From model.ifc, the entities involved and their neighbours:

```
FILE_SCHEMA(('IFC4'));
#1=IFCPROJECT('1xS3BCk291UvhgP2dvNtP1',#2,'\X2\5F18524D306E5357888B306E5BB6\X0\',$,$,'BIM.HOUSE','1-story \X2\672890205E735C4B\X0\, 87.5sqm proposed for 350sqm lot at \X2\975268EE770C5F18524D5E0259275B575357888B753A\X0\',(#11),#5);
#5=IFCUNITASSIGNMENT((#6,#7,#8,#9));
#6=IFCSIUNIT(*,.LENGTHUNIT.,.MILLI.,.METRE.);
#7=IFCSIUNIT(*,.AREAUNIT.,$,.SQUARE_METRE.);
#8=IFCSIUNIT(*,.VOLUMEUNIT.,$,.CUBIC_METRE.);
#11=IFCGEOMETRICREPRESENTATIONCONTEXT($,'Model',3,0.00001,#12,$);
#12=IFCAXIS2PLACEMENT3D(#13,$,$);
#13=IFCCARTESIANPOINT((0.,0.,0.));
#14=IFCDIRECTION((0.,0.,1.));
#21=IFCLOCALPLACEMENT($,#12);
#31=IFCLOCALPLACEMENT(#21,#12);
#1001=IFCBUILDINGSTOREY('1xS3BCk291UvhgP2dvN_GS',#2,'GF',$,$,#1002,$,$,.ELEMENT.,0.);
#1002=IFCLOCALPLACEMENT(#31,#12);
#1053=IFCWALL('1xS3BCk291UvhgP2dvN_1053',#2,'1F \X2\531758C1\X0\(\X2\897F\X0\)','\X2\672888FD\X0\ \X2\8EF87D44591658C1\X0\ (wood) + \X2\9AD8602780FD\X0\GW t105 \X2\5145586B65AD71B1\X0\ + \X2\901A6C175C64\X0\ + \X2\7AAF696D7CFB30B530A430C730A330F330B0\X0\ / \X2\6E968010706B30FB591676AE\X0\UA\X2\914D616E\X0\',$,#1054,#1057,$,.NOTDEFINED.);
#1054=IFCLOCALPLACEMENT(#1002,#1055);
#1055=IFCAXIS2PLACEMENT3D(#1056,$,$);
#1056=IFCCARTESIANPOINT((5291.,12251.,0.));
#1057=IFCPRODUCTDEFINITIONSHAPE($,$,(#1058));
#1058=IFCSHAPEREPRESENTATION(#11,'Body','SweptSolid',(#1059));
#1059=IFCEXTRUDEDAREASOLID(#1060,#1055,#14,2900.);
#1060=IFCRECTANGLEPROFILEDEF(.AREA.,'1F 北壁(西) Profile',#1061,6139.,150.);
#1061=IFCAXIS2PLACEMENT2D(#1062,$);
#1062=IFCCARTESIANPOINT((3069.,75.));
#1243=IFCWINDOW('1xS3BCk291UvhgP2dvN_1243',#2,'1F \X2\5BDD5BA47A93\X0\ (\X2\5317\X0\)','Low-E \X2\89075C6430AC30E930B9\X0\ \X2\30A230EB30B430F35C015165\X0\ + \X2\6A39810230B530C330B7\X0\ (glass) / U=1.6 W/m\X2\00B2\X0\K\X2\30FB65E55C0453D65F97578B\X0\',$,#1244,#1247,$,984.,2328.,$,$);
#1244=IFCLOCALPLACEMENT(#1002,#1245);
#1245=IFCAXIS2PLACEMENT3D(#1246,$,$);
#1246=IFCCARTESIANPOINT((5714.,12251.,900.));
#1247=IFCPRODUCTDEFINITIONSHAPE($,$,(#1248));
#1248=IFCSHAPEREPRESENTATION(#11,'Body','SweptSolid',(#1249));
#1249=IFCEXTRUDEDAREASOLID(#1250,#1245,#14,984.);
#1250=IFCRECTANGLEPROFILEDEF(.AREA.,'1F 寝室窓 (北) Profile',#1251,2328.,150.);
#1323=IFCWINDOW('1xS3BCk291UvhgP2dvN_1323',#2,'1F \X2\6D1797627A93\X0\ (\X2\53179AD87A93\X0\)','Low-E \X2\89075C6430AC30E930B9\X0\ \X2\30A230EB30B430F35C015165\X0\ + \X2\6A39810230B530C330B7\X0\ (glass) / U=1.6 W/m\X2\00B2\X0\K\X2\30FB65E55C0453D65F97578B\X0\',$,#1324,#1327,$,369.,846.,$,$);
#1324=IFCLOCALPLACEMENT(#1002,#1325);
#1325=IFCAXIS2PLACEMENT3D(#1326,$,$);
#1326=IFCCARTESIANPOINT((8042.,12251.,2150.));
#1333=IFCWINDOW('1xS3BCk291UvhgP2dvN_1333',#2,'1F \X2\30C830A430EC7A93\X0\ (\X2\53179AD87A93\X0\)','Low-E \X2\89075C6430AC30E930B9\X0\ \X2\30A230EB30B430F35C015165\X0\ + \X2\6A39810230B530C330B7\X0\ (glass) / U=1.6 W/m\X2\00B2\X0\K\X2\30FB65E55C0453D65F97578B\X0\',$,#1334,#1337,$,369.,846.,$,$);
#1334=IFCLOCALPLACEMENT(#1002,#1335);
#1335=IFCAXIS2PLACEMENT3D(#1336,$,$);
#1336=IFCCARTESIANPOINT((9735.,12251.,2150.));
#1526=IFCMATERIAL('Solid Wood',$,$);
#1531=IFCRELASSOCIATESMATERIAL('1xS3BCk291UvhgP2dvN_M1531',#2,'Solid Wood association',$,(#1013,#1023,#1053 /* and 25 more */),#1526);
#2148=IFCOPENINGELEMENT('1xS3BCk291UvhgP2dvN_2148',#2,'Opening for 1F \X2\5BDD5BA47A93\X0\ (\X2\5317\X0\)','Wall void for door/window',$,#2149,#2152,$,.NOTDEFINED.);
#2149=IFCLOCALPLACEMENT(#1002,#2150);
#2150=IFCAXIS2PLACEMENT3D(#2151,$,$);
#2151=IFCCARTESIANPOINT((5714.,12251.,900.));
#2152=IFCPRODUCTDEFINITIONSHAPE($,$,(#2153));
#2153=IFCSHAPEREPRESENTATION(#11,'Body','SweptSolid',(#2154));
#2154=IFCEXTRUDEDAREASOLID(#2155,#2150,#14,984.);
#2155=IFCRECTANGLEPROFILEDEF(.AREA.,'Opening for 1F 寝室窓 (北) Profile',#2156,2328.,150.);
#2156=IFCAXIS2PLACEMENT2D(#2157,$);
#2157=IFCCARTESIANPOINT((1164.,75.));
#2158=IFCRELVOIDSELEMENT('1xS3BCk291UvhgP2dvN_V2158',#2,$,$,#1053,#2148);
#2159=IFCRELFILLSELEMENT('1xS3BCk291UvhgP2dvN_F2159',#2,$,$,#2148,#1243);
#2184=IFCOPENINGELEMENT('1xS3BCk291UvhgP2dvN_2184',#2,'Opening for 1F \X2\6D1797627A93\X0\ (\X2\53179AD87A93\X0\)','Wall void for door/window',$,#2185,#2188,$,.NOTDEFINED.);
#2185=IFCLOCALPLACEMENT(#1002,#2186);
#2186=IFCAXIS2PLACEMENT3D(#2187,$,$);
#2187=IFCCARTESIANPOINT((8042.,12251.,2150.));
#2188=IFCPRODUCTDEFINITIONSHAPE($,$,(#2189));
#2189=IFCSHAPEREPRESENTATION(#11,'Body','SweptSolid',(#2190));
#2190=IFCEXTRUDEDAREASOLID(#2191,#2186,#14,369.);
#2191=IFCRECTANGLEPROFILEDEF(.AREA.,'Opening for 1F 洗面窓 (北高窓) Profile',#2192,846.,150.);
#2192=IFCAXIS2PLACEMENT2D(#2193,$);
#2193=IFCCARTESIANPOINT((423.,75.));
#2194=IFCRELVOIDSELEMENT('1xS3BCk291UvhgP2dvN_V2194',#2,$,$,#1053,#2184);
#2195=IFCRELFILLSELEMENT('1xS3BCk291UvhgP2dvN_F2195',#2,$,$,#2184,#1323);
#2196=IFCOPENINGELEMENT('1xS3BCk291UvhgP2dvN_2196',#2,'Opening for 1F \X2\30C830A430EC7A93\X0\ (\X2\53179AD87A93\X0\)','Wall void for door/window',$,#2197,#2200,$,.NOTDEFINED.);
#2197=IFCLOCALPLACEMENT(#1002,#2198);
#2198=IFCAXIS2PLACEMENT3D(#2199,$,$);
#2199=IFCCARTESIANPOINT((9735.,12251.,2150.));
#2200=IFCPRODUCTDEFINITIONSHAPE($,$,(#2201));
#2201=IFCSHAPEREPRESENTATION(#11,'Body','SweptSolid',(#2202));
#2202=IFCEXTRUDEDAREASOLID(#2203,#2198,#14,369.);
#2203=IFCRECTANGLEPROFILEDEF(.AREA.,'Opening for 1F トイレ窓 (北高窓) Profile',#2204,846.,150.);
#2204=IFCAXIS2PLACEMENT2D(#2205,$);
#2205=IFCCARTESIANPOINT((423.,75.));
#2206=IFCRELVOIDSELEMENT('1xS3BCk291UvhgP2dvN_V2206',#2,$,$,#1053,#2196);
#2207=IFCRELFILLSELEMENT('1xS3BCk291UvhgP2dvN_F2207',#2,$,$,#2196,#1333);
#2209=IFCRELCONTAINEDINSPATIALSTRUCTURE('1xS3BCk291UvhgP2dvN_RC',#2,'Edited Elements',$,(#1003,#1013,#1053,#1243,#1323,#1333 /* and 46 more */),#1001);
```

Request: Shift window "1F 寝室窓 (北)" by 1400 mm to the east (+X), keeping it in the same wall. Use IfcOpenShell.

```python
import ifcopenshell
import ifcopenshell.api.geometry
import ifcopenshell.util.placement

model = ifcopenshell.open("model.ifc")

window = model.by_guid("1xS3BCk291UvhgP2dvN_1243")
opening = window.FillsVoids[0].RelatingOpeningElement
wall = opening.VoidsElements[0].RelatingBuildingElement

wall_matrix = ifcopenshell.util.placement.get_local_placement(wall.ObjectPlacement)
shift = wall_matrix[:3, 0] * 1400.0
before = ifcopenshell.util.placement.get_local_placement(window.ObjectPlacement)[:3, 3].copy()

# The window is not placed relative to its opening, so move both.
for product in (opening, window):
    matrix = ifcopenshell.util.placement.get_local_placement(product.ObjectPlacement)
    matrix[:3, 3] += shift
    ifcopenshell.api.geometry.edit_object_placement(model, product=product, matrix=matrix, is_si=False)

after = ifcopenshell.util.placement.get_local_placement(window.ObjectPlacement)[:3, 3]
print("window moved by", (after - before).round(3) + 0.0)

model.write("model_edited.ifc")
```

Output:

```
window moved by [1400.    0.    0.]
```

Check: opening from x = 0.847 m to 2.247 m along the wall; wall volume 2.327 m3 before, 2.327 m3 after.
